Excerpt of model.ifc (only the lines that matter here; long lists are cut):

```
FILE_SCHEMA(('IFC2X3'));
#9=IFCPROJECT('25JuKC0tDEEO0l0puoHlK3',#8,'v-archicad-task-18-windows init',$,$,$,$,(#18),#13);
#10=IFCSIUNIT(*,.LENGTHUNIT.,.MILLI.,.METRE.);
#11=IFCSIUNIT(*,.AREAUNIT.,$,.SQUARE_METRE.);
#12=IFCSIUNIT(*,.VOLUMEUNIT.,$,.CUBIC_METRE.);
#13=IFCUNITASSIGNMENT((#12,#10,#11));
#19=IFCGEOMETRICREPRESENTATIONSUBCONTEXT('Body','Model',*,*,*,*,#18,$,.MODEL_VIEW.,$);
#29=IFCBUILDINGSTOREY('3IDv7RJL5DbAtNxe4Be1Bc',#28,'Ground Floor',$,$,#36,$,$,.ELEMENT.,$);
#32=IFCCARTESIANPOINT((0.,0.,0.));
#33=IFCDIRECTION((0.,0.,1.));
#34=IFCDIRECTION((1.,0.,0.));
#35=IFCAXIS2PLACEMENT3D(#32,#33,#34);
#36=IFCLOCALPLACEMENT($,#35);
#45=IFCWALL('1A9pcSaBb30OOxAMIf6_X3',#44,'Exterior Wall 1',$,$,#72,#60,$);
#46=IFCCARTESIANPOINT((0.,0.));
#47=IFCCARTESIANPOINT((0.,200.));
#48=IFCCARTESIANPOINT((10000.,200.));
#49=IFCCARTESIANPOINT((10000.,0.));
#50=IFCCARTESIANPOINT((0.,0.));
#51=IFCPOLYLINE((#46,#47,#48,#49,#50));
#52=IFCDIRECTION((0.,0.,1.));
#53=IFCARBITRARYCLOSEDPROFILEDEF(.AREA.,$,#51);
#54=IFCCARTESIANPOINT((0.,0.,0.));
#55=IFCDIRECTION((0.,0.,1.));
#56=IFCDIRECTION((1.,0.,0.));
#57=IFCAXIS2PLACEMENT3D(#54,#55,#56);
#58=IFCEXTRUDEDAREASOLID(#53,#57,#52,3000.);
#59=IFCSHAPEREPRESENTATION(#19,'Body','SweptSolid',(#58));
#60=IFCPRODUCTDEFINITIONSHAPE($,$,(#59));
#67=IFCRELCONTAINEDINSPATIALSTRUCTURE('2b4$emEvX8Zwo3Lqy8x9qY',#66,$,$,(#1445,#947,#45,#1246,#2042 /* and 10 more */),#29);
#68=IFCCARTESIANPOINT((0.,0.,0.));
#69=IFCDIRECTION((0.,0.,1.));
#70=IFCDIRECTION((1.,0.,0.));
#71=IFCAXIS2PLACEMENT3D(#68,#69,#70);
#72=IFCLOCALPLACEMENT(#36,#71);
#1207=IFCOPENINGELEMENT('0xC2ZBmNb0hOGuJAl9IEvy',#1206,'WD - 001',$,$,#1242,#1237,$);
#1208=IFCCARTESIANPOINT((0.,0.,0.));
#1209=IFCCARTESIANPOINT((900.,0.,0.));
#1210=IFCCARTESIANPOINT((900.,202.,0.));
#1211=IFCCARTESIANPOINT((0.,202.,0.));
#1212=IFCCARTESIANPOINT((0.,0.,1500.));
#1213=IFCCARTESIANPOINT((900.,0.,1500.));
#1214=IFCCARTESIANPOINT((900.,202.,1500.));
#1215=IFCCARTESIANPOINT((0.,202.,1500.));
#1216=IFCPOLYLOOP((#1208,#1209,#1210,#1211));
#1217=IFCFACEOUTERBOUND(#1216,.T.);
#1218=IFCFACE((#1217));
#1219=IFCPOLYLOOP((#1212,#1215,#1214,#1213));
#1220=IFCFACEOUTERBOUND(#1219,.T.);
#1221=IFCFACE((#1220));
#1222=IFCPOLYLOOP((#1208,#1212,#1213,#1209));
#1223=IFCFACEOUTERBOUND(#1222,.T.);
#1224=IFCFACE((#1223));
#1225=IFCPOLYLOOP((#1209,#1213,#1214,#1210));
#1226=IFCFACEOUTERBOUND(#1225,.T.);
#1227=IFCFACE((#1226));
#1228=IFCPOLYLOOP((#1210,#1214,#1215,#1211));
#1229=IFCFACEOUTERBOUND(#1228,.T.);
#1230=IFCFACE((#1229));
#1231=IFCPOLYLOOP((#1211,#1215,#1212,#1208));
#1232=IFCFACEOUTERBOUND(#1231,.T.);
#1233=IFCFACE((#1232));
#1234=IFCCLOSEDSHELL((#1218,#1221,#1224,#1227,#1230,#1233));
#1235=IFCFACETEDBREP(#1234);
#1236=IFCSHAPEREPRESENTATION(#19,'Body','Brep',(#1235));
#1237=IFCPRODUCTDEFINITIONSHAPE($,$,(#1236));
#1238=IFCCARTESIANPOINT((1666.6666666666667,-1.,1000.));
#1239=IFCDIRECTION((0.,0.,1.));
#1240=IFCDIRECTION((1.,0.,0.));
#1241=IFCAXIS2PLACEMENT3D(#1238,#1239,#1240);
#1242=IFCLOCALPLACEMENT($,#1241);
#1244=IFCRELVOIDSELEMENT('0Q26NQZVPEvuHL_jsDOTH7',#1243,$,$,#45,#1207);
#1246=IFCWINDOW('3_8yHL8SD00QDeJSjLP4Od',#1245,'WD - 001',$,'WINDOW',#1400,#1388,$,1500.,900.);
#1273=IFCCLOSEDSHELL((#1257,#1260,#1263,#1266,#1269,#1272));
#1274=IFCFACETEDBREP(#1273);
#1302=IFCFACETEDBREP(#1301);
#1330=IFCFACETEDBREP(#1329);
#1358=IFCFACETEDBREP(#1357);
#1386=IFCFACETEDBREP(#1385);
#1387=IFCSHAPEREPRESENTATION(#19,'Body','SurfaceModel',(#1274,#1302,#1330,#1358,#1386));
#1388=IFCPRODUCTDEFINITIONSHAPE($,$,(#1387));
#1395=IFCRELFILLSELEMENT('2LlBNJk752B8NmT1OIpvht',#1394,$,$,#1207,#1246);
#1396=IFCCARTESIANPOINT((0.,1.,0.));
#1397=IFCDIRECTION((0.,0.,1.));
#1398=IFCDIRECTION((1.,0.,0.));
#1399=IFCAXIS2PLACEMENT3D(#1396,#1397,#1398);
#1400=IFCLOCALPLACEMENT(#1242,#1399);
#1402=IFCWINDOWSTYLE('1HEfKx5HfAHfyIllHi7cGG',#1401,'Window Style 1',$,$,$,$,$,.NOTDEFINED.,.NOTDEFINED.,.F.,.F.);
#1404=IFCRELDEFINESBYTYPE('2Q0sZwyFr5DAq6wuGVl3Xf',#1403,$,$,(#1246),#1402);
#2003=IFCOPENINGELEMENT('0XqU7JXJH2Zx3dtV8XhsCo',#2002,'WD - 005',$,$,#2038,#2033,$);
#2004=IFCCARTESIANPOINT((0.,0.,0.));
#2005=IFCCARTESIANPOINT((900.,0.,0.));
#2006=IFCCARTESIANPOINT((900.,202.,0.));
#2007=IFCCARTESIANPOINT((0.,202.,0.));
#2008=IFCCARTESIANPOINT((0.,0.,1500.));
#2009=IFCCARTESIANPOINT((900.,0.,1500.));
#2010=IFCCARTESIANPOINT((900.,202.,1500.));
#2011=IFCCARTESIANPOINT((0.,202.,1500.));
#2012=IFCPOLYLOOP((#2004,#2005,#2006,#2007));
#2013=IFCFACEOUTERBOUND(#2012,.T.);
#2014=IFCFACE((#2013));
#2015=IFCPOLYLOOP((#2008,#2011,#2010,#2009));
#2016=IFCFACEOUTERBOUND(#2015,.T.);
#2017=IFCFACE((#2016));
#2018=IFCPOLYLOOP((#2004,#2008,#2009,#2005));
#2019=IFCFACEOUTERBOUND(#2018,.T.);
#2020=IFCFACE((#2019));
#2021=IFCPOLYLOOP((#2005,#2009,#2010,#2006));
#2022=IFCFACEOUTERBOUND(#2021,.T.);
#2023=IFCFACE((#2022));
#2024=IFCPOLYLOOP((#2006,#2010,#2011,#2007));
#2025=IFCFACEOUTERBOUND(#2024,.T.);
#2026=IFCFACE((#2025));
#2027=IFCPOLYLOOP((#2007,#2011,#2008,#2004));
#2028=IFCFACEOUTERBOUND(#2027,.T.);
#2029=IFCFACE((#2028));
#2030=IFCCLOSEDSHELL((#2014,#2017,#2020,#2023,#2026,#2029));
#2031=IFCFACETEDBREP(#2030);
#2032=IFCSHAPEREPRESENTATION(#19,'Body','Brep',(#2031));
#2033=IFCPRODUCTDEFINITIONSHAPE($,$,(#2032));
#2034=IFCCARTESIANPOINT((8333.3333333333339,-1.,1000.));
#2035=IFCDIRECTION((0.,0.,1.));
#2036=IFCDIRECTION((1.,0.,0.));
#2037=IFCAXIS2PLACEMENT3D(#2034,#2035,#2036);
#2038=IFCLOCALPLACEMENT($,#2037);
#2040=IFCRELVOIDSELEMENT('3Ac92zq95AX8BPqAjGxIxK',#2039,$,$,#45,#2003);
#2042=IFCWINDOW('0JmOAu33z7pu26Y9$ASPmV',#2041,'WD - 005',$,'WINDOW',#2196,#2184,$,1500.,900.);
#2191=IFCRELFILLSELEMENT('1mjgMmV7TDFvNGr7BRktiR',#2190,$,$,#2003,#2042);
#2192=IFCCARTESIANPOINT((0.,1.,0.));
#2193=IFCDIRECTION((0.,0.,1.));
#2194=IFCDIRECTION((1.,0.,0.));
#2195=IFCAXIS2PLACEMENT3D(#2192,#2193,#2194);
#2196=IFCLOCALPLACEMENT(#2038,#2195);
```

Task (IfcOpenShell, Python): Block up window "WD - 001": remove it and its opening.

```python
import ifcopenshell
import ifcopenshell.api.feature
import ifcopenshell.api.root
import ifcopenshell.geom
import ifcopenshell.util.shape

model = ifcopenshell.open("model.ifc")
settings = ifcopenshell.geom.settings()


def volume(element):
    """Net volume in cubic metres, openings subtracted."""
    shape = ifcopenshell.geom.create_shape(settings, element)
    return ifcopenshell.util.shape.get_volume(shape.geometry)


window = model.by_id(1246)
opening = window.FillsVoids[0].RelatingOpeningElement
wall = opening.VoidsElements[0].RelatingBuildingElement
before = volume(wall)

ifcopenshell.api.root.remove_product(model, product=window)
ifcopenshell.api.feature.remove_feature(model, feature=opening)

after = volume(wall)

print(f"wall volume {before:.3f} -> {after:.3f} m3")

model.write("model_edited.ifc")
```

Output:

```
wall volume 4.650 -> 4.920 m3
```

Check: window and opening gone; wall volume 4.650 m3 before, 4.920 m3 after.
